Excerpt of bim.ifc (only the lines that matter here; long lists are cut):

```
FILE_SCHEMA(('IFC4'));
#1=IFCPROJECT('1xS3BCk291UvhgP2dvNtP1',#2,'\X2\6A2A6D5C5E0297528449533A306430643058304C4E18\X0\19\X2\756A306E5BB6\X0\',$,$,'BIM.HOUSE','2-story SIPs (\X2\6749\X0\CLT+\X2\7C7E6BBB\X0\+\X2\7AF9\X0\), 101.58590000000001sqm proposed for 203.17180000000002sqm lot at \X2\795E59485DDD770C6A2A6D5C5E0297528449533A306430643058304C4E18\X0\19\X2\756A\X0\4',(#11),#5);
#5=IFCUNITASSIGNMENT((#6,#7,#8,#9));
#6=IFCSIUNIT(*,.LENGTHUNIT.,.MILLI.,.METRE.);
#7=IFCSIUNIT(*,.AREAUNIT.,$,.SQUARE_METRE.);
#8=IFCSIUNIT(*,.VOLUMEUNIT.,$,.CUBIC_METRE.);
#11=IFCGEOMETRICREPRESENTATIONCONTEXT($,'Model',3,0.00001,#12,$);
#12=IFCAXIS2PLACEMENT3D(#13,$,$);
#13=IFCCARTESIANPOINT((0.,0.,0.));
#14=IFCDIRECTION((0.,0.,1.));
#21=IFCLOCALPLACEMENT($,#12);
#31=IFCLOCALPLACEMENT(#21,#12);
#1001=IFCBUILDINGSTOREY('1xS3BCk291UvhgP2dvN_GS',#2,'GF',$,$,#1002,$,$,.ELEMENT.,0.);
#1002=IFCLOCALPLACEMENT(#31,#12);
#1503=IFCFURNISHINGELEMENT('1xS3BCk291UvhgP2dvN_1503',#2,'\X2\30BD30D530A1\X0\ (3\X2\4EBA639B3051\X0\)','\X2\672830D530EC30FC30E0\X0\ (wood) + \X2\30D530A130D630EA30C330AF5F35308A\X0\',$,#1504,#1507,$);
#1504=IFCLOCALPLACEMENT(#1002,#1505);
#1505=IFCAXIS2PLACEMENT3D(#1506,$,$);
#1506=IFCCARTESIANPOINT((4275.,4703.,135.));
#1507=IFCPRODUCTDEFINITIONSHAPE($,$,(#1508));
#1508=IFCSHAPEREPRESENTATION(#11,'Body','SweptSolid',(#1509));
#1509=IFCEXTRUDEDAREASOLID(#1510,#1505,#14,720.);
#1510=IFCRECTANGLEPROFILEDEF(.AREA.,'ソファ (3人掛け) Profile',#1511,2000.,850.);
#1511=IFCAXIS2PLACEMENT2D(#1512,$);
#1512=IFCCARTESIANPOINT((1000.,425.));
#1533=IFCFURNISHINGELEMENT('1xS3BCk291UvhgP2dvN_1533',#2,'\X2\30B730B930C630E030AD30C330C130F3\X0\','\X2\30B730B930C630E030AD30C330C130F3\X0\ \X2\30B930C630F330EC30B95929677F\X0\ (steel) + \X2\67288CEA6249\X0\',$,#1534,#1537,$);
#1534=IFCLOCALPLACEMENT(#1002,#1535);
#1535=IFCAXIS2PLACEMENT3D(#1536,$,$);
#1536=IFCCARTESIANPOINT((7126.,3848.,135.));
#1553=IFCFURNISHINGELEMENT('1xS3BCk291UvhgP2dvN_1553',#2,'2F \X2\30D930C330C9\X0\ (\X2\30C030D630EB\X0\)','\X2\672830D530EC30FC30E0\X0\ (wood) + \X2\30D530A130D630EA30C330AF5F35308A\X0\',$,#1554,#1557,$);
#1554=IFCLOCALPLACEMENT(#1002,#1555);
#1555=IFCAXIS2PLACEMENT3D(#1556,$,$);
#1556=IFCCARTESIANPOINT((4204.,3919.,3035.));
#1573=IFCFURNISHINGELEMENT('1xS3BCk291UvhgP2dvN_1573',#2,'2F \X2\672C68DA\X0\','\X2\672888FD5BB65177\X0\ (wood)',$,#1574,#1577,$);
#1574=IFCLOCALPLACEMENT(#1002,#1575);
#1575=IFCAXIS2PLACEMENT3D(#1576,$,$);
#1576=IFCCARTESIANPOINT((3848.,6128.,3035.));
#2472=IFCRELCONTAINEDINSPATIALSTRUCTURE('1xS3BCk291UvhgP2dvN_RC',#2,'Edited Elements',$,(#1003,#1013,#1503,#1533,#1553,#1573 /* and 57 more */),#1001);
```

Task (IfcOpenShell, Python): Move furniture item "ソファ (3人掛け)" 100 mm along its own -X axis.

```python
import ifcopenshell
import ifcopenshell.api.geometry
import ifcopenshell.util.placement
import ifcopenshell.util.unit

model = ifcopenshell.open("bim.ifc")
unit_scale = ifcopenshell.util.unit.calculate_unit_scale(model)

item = model.by_id(1503)
matrix = ifcopenshell.util.placement.get_local_placement(item.ObjectPlacement)
matrix[:3, 3] -= matrix[:3, 0] * 0.1 / unit_scale
ifcopenshell.api.geometry.edit_object_placement(model, product=item, matrix=matrix, is_si=False)

print(ifcopenshell.util.placement.get_local_placement(item.ObjectPlacement).round(3) + 0.0)

model.write("bim_updated.ifc")
```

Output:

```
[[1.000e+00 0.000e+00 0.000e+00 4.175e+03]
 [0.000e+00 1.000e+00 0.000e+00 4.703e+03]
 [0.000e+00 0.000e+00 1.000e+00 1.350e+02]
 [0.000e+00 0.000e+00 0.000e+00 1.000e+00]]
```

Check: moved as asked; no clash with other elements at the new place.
